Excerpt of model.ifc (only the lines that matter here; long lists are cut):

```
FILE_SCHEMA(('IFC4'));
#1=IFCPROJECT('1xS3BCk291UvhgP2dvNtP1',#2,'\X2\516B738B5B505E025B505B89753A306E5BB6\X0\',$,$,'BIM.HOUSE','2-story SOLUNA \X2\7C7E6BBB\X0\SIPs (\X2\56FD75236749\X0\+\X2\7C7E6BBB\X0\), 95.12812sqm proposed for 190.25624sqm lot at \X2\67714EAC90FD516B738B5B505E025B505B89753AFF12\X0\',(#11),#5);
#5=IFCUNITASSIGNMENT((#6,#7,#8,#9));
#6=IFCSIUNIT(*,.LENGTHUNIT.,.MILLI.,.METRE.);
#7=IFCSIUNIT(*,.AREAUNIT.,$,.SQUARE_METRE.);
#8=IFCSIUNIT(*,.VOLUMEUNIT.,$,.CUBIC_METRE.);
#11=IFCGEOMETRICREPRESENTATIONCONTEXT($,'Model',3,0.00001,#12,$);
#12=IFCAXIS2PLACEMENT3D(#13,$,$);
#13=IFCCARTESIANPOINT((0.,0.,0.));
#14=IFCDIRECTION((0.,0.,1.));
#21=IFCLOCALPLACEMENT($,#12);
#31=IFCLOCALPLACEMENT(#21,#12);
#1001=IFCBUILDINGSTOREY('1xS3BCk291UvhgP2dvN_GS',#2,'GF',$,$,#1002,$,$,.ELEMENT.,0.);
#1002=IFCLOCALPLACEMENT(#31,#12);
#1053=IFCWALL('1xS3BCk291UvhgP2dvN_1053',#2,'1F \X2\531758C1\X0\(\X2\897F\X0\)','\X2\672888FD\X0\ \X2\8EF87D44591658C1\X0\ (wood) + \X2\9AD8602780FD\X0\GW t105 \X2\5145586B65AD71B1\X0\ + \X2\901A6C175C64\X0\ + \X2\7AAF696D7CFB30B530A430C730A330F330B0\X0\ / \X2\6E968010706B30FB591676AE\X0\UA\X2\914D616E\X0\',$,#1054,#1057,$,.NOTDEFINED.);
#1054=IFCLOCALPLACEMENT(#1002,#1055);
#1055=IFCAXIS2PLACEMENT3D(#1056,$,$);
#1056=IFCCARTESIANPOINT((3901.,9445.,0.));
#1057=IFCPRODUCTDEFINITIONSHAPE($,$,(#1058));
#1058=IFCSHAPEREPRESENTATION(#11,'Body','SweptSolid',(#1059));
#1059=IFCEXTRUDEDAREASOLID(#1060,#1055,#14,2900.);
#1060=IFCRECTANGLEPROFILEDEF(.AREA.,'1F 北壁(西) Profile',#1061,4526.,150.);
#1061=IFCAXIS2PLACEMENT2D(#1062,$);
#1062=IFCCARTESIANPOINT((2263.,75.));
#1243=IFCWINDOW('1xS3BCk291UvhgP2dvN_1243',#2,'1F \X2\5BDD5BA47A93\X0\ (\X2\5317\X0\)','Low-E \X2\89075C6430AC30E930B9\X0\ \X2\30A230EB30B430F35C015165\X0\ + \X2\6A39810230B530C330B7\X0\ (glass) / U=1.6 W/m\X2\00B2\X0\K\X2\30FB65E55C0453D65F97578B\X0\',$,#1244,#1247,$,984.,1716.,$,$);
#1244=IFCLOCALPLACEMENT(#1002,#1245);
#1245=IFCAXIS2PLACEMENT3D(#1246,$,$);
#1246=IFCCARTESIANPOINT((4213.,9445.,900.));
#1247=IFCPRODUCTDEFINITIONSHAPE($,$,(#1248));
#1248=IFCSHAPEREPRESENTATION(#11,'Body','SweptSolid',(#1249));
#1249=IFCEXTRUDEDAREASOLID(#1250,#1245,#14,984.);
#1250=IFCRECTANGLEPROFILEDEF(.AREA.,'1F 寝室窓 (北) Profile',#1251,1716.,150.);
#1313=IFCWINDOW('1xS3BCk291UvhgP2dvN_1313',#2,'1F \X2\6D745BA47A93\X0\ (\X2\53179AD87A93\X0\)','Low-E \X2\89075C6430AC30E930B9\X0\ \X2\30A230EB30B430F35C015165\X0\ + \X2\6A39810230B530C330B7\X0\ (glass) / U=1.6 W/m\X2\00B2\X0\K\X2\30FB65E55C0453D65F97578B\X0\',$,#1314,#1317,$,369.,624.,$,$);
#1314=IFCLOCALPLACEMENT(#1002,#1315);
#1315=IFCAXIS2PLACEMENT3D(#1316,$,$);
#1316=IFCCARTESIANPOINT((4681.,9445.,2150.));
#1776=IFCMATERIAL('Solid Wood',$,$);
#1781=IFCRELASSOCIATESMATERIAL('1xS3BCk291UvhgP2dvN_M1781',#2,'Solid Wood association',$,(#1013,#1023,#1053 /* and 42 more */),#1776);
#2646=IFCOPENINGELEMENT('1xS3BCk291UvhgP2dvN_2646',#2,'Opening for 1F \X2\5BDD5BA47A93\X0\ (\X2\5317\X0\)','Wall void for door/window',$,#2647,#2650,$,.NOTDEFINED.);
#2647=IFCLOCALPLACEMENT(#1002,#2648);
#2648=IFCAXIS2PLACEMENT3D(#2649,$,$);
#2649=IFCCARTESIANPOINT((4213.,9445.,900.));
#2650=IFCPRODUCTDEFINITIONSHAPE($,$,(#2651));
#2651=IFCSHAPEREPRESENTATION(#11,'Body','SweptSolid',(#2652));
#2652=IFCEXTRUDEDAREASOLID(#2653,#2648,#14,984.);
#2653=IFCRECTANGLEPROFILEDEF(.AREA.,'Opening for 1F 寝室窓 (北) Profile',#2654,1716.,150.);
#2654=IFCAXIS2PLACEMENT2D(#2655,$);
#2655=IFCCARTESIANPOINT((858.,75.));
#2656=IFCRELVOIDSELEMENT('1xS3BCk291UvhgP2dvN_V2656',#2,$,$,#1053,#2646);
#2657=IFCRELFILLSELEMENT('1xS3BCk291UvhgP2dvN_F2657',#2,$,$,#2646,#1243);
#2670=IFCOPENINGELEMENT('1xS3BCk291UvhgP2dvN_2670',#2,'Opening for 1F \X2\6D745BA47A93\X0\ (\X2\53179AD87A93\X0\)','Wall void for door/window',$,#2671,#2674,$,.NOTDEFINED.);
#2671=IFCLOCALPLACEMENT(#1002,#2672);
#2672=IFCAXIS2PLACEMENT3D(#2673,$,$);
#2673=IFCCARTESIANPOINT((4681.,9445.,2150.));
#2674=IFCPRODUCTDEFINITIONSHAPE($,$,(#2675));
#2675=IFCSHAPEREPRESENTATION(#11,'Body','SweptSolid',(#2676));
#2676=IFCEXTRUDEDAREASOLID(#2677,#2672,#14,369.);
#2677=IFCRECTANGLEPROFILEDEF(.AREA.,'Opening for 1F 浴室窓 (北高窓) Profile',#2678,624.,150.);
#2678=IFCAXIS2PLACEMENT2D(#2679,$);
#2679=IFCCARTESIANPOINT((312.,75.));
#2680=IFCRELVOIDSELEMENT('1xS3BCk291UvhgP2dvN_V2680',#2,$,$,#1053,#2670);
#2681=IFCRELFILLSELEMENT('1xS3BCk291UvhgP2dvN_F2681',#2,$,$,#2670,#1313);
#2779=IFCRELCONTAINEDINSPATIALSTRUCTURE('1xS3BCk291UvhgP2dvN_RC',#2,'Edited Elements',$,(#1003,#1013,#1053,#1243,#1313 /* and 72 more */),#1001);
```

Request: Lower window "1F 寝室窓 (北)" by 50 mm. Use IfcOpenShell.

```python
import numpy as np
import ifcopenshell
import ifcopenshell.api.geometry
import ifcopenshell.util.placement
import ifcopenshell.util.unit

model = ifcopenshell.open("model.ifc")
unit_scale = ifcopenshell.util.unit.calculate_unit_scale(model)

window = model.by_guid("1xS3BCk291UvhgP2dvN_1243")
opening = window.FillsVoids[0].RelatingOpeningElement
dz = -0.05 / unit_scale

shift = np.array([0.0, 0.0, dz])
# The window is not placed relative to its opening, so move both.
for product in (opening, window):
    matrix = ifcopenshell.util.placement.get_local_placement(product.ObjectPlacement)
    matrix[:3, 3] += shift
    ifcopenshell.api.geometry.edit_object_placement(model, product=product, matrix=matrix, is_si=False)

print(f"moved by {dz * unit_scale:+.3f} m")

model.write("model_updated.ifc")
```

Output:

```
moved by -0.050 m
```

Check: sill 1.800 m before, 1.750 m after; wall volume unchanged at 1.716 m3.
